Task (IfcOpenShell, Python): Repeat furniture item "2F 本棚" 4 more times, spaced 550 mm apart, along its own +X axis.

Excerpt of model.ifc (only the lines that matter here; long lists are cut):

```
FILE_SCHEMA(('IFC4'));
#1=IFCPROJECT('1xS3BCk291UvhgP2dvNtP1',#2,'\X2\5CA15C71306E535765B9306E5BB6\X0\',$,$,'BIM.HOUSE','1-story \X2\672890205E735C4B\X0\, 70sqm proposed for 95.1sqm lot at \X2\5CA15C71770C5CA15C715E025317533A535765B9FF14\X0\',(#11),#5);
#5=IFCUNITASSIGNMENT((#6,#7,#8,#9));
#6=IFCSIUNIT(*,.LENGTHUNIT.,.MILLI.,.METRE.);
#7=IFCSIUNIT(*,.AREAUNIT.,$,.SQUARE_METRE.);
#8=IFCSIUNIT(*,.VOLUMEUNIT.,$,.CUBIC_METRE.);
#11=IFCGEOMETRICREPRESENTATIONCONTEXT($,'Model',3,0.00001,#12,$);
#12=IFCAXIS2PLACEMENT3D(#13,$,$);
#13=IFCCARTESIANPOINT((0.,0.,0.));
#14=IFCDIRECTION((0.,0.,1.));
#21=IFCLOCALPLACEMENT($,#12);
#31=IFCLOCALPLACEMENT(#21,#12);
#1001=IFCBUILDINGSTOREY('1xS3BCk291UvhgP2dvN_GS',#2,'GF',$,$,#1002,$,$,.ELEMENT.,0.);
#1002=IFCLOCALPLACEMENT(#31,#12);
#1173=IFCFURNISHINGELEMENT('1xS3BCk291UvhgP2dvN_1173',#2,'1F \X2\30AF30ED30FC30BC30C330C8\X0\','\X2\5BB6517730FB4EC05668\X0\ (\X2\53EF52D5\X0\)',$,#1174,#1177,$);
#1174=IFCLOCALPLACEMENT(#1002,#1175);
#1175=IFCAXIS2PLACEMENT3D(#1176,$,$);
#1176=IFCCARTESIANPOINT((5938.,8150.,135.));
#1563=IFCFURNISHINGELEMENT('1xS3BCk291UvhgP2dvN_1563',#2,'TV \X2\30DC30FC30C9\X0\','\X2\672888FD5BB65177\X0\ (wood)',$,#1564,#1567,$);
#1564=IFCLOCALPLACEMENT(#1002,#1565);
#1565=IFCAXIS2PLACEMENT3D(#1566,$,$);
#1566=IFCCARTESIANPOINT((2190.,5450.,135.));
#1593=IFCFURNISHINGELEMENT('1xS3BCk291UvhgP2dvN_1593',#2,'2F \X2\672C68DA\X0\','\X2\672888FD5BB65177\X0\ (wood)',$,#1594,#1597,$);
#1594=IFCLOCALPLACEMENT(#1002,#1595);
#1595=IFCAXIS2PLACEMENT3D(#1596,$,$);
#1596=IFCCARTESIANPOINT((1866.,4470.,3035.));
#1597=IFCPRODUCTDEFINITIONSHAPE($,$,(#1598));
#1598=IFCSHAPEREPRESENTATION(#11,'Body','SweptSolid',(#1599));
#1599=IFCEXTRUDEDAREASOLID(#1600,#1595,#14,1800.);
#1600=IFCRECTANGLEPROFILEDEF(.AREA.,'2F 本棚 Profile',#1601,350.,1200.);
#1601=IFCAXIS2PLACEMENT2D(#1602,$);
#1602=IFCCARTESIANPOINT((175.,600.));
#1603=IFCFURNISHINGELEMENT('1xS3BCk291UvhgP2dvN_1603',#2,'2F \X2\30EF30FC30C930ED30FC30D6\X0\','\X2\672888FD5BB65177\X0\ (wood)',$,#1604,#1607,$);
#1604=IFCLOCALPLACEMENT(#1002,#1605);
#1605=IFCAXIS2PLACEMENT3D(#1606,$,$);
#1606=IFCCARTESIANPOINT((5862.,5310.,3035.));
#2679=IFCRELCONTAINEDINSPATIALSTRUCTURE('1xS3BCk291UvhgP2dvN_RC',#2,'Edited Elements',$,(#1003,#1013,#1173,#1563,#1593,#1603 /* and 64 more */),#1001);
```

```python
import ifcopenshell
import ifcopenshell.api.geometry
import ifcopenshell.api.root
import ifcopenshell.util.element
import ifcopenshell.util.placement

model = ifcopenshell.open("model.ifc")


def reuse_history(source, copy):
    """copy_class also copies each property set's owner history, people and application; keep the originals."""
    for rel in copy.IsDefinedBy:
        if rel.is_a("IfcRelDefinesByProperties") and (history := rel.RelatingPropertyDefinition.OwnerHistory):
            rel.RelatingPropertyDefinition.OwnerHistory = source.OwnerHistory
            ifcopenshell.util.element.remove_deep2(model, history)


source = model.by_id(1593)
base = ifcopenshell.util.placement.get_local_placement(source.ObjectPlacement)
step = base[:3, 0] * 550.0

for i in range(1, 5):
    copy = ifcopenshell.api.root.copy_class(model, product=source)
    copy.Representation = ifcopenshell.util.element.copy_deep(
        model, source.Representation, exclude=["IfcGeometricRepresentationContext", "IfcRepresentationMap"]
    )
    reuse_history(source, copy)
    matrix = base.copy()
    matrix[:3, 3] += i * step
    print("added at", matrix[:3, 3].round(3) + 0.0)
    ifcopenshell.api.geometry.edit_object_placement(model, product=copy, matrix=matrix, is_si=False)

model.write("model-out.ifc")
```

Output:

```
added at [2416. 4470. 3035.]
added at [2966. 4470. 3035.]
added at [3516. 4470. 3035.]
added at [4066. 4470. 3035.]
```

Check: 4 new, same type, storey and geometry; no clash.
